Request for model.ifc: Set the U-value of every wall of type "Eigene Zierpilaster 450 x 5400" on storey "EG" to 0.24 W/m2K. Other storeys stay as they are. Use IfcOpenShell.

First a look at what the model holds.

```python
import ifcopenshell
import ifcopenshell.util.element

model = ifcopenshell.open("model.ifc")
print(model.schema)
storey = next(s for s in model.by_type("IfcBuildingStorey") if s.Name == "EG")
walls = [e for e in ifcopenshell.util.element.get_decomposition(storey) if e.is_a("IfcWall")]
seen = {}
for e in walls:
    element_type = ifcopenshell.util.element.get_type(e)
    key = (element_type.Name if element_type != e and element_type else None, ifcopenshell.util.element.get_pset(e, "Pset_WallCommon", "ThermalTransmittance"))
    seen[key] = seen.get(key, 0) + 1
for (name, value), count in sorted(seen.items(), key=str):
    print(count, "x", name, "|", value)
```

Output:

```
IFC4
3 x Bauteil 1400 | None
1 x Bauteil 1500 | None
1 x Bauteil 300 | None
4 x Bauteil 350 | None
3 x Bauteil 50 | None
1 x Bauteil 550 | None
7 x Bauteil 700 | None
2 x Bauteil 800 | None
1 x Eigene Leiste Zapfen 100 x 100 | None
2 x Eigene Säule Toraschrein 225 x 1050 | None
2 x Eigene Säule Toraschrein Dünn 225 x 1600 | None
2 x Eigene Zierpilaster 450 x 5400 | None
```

```python
import ifcopenshell
import ifcopenshell.api.pset
import ifcopenshell.util.element

model = ifcopenshell.open("model.ifc")

storey = next(s for s in model.by_type("IfcBuildingStorey") if s.Name == "EG")
walls = [e for e in ifcopenshell.util.element.get_decomposition(storey) if e.is_a("IfcWall")]

count = 0
for e in walls:
    element_type = ifcopenshell.util.element.get_type(e)
    if element_type in (None, e) or element_type.Name != "Eigene Zierpilaster 450 x 5400":
        continue
    # add_pset returns the element's existing set when there is one.
    pset = ifcopenshell.api.pset.add_pset(model, product=e, name="Pset_WallCommon")
    ifcopenshell.api.pset.edit_pset(model, pset=pset, properties={"ThermalTransmittance": 0.24})
    count += 1

print(count, "walls updated")

model.write("model_edited.ifc")
```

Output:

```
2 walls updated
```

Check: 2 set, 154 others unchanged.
